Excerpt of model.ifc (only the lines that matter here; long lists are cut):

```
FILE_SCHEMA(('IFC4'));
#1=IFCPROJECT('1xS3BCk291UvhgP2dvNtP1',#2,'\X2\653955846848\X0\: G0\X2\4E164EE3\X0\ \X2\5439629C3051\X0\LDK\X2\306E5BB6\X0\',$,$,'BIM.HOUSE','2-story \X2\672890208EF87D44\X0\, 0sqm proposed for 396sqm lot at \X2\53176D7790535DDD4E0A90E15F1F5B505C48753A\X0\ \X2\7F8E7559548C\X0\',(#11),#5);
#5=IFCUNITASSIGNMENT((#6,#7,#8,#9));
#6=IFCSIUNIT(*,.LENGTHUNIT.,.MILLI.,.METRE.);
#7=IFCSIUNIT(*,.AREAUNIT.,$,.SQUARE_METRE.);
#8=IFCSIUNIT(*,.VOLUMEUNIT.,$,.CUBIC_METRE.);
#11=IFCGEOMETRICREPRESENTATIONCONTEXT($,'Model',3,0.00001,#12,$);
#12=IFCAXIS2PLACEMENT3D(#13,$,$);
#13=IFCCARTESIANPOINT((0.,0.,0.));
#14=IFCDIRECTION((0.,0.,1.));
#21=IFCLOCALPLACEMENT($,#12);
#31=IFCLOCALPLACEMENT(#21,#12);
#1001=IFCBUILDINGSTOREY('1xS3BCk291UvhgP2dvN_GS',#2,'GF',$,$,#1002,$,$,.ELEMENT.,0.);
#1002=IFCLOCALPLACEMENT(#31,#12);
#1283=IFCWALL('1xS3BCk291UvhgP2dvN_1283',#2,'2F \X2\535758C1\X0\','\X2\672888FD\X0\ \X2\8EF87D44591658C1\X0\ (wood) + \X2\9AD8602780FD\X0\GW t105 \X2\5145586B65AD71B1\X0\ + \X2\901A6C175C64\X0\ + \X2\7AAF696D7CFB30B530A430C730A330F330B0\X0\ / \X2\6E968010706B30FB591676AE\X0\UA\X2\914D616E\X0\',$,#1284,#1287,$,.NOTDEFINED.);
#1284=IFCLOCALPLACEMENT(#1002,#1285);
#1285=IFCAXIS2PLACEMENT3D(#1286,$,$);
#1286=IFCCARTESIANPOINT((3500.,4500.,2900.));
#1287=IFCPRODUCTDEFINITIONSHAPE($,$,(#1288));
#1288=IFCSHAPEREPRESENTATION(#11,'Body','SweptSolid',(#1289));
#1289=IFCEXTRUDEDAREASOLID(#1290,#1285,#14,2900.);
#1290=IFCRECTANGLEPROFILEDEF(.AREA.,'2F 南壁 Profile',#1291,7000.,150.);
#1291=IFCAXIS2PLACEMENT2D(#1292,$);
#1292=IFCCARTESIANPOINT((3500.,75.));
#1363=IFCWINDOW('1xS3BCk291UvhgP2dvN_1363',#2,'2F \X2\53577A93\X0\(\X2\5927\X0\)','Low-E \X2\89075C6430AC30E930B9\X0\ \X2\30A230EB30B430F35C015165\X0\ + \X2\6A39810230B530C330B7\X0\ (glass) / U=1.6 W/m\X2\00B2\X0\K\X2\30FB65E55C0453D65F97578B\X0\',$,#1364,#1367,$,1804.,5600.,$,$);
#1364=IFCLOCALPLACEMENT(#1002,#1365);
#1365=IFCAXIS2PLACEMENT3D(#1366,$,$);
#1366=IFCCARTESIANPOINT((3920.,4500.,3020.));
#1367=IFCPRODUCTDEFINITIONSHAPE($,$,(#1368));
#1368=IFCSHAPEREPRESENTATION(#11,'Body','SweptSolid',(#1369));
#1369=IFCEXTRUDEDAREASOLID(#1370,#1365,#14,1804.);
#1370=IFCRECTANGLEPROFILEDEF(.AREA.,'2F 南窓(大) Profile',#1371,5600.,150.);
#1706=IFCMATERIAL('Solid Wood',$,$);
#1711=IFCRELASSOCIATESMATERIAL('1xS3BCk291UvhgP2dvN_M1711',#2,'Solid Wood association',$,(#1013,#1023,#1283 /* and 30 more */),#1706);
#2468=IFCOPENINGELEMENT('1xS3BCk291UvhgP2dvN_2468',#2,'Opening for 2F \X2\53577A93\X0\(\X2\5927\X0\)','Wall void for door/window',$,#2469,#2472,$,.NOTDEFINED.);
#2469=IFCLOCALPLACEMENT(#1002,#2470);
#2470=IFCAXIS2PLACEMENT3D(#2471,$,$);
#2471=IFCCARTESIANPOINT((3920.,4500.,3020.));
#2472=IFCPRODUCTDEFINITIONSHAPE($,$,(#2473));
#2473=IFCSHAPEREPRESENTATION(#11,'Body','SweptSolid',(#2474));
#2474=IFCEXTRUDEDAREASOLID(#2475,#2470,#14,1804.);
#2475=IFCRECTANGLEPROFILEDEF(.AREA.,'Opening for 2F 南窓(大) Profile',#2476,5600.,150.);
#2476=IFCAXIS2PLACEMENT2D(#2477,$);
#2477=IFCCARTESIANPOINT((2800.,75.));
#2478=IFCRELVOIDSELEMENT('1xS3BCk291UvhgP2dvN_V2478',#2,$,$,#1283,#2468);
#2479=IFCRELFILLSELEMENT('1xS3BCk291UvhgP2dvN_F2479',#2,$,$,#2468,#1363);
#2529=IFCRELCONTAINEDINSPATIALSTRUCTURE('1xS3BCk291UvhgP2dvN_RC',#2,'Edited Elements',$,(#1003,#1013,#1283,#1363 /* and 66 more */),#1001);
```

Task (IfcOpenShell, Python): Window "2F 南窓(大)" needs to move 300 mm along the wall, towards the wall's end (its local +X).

```python
import ifcopenshell
import ifcopenshell.api.geometry
import ifcopenshell.util.placement

model = ifcopenshell.open("model.ifc")

window = model.by_guid("1xS3BCk291UvhgP2dvN_1363")
opening = window.FillsVoids[0].RelatingOpeningElement
wall = opening.VoidsElements[0].RelatingBuildingElement

wall_matrix = ifcopenshell.util.placement.get_local_placement(wall.ObjectPlacement)
shift = wall_matrix[:3, 0] * 300.0
before = ifcopenshell.util.placement.get_local_placement(window.ObjectPlacement)[:3, 3].copy()

# The window is not placed relative to its opening, so move both.
for product in (opening, window):
    matrix = ifcopenshell.util.placement.get_local_placement(product.ObjectPlacement)
    matrix[:3, 3] += shift
    ifcopenshell.api.geometry.edit_object_placement(model, product=product, matrix=matrix, is_si=False)

after = ifcopenshell.util.placement.get_local_placement(window.ObjectPlacement)[:3, 3]
print("window moved by", (after - before).round(3) + 0.0)

model.write("model_edited.ifc")
```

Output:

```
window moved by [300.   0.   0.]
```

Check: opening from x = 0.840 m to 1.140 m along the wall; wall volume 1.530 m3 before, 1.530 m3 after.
